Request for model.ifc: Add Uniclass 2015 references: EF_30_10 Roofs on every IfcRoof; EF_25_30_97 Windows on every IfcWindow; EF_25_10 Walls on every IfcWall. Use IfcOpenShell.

First a look at what the model holds.

```python
import ifcopenshell

model = ifcopenshell.open("model.ifc")
print(model.schema)
print("classifications:", [c.Name for c in model.by_type("IfcClassification")])
for ifc_class in ("IfcDoor", "IfcRoof", "IfcStair", "IfcWall", "IfcWindow"):
    print(ifc_class, len(model.by_type(ifc_class)))
```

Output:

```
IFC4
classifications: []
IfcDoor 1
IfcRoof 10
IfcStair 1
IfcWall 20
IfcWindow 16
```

```python
import ifcopenshell
import ifcopenshell.api.classification

model = ifcopenshell.open("model.ifc")

system = ifcopenshell.api.classification.add_classification(model, classification="Uniclass 2015")

codes = {
    "IfcRoof": ("EF_30_10", "Roofs"),
    "IfcWindow": ("EF_25_30_97", "Windows"),
    "IfcWall": ("EF_25_10", "Walls"),
}
for ifc_class, (code, name) in codes.items():
    products = model.by_type(ifc_class)
    ifcopenshell.api.classification.add_reference(
        model, products=products, classification=system, identification=code, name=name
    )
    print(code, len(products))

model.write("model_updated.ifc")
```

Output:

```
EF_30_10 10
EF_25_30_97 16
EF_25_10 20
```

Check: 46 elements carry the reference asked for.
